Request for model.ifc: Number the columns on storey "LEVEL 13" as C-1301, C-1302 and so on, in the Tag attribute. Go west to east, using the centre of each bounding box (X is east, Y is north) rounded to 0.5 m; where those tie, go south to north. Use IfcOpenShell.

First a look at what the model holds.

```python
import ifcopenshell
import ifcopenshell.util.element
import ifcopenshell.util.placement

model = ifcopenshell.open("model.ifc")
print(model.schema)
storey = next(s for s in model.by_type("IfcBuildingStorey") if s.Name == "LEVEL 13")
columns = [e for e in ifcopenshell.util.element.get_decomposition(storey) if e.is_a("IfcColumn")]
for e in sorted(columns, key=lambda e: e.id()):
    origin = ifcopenshell.util.placement.get_local_placement(e.ObjectPlacement)[:3, 3]
    print(e.id(), e.Tag, e.Name, origin.round(2) + 0.0, sep=" | ")
```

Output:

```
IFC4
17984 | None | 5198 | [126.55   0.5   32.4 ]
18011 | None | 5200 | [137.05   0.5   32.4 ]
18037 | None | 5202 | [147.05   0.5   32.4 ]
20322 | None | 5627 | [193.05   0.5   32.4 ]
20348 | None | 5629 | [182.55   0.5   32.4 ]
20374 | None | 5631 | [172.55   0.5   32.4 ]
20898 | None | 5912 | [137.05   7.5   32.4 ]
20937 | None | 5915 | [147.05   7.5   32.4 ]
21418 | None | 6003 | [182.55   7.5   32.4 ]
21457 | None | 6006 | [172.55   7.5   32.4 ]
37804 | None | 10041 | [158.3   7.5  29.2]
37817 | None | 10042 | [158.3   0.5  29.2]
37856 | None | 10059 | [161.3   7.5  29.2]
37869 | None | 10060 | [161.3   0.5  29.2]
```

```python
import ifcopenshell
import ifcopenshell.geom
import ifcopenshell.util.element
import ifcopenshell.util.shape

model = ifcopenshell.open("model.ifc")
settings = ifcopenshell.geom.settings()
settings.set("use-world-coords", True)


def centre(element):
    shape = ifcopenshell.geom.create_shape(settings, element)
    return ifcopenshell.util.shape.get_bbox_centroid(shape.geometry)


storey = next(s for s in model.by_type("IfcBuildingStorey") if s.Name == "LEVEL 13")
columns = [e for e in ifcopenshell.util.element.get_decomposition(storey) if e.is_a("IfcColumn")]

# Insertion points can sit at a corner or the storey origin, so sort by the geometry (in metres).
centres = {e: centre(e) for e in columns}
columns.sort(key=lambda e: (round(centres[e][0] / 0.5), centres[e][1]))

for i, e in enumerate(columns, start=1):
    number = f"C-13{i:02d}"
    e.Tag = number
    print(e.id(), number)

model.write("model_updated.ifc")
```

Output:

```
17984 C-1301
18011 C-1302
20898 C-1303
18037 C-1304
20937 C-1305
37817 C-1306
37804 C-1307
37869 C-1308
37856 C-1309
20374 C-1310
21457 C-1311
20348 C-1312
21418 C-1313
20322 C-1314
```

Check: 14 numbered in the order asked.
